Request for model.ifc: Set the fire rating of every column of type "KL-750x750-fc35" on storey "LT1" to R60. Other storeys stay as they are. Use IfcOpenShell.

First a look at what the model holds.

```python
import ifcopenshell
import ifcopenshell.util.element

model = ifcopenshell.open("model.ifc")
print(model.schema)
storey = next(s for s in model.by_type("IfcBuildingStorey") if s.Name == "LT1")
columns = [e for e in ifcopenshell.util.element.get_decomposition(storey) if e.is_a("IfcColumn")]
seen = {}
for e in columns:
    element_type = ifcopenshell.util.element.get_type(e)
    key = (element_type.Name if element_type != e and element_type else None, ifcopenshell.util.element.get_pset(e, "Pset_ColumnCommon", "FireRating"))
    seen[key] = seen.get(key, 0) + 1
for (name, value), count in sorted(seen.items(), key=str):
    print(count, "x", name, "|", value)
```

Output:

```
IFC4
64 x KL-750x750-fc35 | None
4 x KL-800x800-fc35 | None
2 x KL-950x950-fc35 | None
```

```python
import ifcopenshell
import ifcopenshell.api.pset
import ifcopenshell.util.element

model = ifcopenshell.open("model.ifc")

storey = next(s for s in model.by_type("IfcBuildingStorey") if s.Name == "LT1")
columns = [e for e in ifcopenshell.util.element.get_decomposition(storey) if e.is_a("IfcColumn")]

count = 0
for e in columns:
    element_type = ifcopenshell.util.element.get_type(e)
    if element_type in (None, e) or element_type.Name != "KL-750x750-fc35":
        continue
    # add_pset returns the element's existing set when there is one.
    pset = ifcopenshell.api.pset.add_pset(model, product=e, name="Pset_ColumnCommon")
    ifcopenshell.api.pset.edit_pset(model, pset=pset, properties={"FireRating": "R60"})
    count += 1

print(count, "columns updated")

model.write("model_edited.ifc")
```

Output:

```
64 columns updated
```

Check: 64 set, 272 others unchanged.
